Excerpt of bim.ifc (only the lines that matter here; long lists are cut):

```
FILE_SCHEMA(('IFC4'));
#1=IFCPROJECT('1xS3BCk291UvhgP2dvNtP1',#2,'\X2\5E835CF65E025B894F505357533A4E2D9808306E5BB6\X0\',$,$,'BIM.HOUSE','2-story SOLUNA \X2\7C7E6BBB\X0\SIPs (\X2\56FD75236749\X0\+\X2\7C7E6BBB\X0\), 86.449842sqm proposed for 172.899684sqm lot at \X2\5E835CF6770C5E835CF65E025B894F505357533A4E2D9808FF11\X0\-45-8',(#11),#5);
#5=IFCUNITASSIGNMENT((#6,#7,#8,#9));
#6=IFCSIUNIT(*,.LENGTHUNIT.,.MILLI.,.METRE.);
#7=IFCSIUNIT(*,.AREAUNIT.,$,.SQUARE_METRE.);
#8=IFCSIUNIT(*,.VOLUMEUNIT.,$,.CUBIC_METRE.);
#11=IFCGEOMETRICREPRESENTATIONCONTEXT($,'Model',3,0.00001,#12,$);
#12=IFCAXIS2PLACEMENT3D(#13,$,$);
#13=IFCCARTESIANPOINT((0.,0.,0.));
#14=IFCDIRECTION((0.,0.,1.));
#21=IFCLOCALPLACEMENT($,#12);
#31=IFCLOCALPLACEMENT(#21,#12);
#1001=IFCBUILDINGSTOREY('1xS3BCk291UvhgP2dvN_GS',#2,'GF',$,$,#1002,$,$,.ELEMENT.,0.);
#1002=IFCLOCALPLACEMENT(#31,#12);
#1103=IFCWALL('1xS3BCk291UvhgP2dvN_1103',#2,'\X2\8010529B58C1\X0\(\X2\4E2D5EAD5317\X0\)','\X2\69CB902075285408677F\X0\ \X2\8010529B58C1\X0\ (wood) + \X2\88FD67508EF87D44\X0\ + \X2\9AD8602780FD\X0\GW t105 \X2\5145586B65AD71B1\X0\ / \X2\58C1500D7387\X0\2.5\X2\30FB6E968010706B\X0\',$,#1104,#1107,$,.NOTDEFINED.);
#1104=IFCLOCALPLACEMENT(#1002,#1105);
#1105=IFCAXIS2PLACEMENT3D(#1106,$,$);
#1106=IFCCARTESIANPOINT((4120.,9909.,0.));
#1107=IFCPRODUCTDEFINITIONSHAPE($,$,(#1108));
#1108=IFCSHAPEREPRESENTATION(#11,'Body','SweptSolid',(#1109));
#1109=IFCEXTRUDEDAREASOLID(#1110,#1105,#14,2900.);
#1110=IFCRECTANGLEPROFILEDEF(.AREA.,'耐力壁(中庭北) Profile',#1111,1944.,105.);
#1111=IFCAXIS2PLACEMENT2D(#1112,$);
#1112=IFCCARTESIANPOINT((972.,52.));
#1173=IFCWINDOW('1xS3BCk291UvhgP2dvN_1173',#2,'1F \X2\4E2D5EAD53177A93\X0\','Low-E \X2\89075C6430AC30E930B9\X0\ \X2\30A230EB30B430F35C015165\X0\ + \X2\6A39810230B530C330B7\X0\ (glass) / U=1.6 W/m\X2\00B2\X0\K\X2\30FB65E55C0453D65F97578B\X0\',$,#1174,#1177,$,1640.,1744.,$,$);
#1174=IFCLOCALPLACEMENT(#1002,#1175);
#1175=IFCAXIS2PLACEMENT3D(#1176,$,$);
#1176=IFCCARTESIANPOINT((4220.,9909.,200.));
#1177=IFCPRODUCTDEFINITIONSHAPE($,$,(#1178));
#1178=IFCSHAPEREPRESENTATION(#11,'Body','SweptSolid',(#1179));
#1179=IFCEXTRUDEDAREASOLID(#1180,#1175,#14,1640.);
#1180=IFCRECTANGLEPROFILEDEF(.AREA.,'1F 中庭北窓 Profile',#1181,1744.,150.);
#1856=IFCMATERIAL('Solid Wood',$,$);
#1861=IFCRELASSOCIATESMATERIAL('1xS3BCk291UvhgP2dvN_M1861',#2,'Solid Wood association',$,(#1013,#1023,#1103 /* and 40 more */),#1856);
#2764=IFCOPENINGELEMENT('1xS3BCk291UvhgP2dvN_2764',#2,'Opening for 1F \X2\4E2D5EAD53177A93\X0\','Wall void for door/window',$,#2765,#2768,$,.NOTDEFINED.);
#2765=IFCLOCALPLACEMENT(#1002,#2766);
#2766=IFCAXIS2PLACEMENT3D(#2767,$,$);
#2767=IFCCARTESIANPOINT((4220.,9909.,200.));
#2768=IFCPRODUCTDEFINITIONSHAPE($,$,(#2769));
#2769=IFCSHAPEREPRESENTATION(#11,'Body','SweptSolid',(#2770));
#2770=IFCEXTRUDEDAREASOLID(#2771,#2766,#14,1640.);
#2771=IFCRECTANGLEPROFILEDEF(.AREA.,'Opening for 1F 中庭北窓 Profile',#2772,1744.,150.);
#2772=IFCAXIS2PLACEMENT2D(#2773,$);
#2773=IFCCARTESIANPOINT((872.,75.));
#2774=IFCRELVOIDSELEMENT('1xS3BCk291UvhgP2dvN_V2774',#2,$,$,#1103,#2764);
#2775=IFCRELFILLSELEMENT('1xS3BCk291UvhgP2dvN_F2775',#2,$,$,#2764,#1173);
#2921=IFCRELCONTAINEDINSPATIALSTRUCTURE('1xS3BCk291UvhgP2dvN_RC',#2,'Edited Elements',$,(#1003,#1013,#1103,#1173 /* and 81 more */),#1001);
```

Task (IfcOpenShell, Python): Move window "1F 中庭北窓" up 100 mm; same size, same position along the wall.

```python
import numpy as np
import ifcopenshell
import ifcopenshell.api.geometry
import ifcopenshell.util.placement
import ifcopenshell.util.unit

model = ifcopenshell.open("bim.ifc")
unit_scale = ifcopenshell.util.unit.calculate_unit_scale(model)

window = model.by_guid("1xS3BCk291UvhgP2dvN_1173")
opening = window.FillsVoids[0].RelatingOpeningElement
dz = 0.1 / unit_scale

shift = np.array([0.0, 0.0, dz])
# The window is not placed relative to its opening, so move both.
for product in (opening, window):
    matrix = ifcopenshell.util.placement.get_local_placement(product.ObjectPlacement)
    matrix[:3, 3] += shift
    ifcopenshell.api.geometry.edit_object_placement(model, product=product, matrix=matrix, is_si=False)

print(f"moved by {dz * unit_scale:+.3f} m")

model.write("bim_rev.ifc")
```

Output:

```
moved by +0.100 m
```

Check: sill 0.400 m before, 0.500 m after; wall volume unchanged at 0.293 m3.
